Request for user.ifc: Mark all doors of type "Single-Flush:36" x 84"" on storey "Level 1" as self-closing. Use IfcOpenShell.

First a look at what the model holds.

```python
import ifcopenshell
import ifcopenshell.util.element

model = ifcopenshell.open("user.ifc")
print(model.schema)
storey = next(s for s in model.by_type("IfcBuildingStorey") if s.Name == "Level 1")
doors = [e for e in ifcopenshell.util.element.get_decomposition(storey) if e.is_a("IfcDoor")]
seen = {}
for e in doors:
    element_type = ifcopenshell.util.element.get_type(e)
    key = (element_type.Name if element_type != e and element_type else None, ifcopenshell.util.element.get_pset(e, "Pset_DoorCommon", "SelfClosing"))
    seen[key] = seen.get(key, 0) + 1
for (name, value), count in sorted(seen.items(), key=str):
    print(count, "x", name, "|", value)
```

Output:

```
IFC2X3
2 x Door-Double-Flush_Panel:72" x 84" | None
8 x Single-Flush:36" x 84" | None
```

```python
import ifcopenshell
import ifcopenshell.api.pset
import ifcopenshell.util.element

model = ifcopenshell.open("user.ifc")

storey = next(s for s in model.by_type("IfcBuildingStorey") if s.Name == "Level 1")
doors = [e for e in ifcopenshell.util.element.get_decomposition(storey) if e.is_a("IfcDoor")]

count = 0
for e in doors:
    element_type = ifcopenshell.util.element.get_type(e)
    if element_type in (None, e) or element_type.Name != 'Single-Flush:36" x 84"':
        continue
    # add_pset returns the element's existing set when there is one.
    pset = ifcopenshell.api.pset.add_pset(model, product=e, name="Pset_DoorCommon")
    ifcopenshell.api.pset.edit_pset(model, pset=pset, properties={"SelfClosing": True})
    count += 1

print(count, "doors updated")

model.write("user_updated.ifc")
```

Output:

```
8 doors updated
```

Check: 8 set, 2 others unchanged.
